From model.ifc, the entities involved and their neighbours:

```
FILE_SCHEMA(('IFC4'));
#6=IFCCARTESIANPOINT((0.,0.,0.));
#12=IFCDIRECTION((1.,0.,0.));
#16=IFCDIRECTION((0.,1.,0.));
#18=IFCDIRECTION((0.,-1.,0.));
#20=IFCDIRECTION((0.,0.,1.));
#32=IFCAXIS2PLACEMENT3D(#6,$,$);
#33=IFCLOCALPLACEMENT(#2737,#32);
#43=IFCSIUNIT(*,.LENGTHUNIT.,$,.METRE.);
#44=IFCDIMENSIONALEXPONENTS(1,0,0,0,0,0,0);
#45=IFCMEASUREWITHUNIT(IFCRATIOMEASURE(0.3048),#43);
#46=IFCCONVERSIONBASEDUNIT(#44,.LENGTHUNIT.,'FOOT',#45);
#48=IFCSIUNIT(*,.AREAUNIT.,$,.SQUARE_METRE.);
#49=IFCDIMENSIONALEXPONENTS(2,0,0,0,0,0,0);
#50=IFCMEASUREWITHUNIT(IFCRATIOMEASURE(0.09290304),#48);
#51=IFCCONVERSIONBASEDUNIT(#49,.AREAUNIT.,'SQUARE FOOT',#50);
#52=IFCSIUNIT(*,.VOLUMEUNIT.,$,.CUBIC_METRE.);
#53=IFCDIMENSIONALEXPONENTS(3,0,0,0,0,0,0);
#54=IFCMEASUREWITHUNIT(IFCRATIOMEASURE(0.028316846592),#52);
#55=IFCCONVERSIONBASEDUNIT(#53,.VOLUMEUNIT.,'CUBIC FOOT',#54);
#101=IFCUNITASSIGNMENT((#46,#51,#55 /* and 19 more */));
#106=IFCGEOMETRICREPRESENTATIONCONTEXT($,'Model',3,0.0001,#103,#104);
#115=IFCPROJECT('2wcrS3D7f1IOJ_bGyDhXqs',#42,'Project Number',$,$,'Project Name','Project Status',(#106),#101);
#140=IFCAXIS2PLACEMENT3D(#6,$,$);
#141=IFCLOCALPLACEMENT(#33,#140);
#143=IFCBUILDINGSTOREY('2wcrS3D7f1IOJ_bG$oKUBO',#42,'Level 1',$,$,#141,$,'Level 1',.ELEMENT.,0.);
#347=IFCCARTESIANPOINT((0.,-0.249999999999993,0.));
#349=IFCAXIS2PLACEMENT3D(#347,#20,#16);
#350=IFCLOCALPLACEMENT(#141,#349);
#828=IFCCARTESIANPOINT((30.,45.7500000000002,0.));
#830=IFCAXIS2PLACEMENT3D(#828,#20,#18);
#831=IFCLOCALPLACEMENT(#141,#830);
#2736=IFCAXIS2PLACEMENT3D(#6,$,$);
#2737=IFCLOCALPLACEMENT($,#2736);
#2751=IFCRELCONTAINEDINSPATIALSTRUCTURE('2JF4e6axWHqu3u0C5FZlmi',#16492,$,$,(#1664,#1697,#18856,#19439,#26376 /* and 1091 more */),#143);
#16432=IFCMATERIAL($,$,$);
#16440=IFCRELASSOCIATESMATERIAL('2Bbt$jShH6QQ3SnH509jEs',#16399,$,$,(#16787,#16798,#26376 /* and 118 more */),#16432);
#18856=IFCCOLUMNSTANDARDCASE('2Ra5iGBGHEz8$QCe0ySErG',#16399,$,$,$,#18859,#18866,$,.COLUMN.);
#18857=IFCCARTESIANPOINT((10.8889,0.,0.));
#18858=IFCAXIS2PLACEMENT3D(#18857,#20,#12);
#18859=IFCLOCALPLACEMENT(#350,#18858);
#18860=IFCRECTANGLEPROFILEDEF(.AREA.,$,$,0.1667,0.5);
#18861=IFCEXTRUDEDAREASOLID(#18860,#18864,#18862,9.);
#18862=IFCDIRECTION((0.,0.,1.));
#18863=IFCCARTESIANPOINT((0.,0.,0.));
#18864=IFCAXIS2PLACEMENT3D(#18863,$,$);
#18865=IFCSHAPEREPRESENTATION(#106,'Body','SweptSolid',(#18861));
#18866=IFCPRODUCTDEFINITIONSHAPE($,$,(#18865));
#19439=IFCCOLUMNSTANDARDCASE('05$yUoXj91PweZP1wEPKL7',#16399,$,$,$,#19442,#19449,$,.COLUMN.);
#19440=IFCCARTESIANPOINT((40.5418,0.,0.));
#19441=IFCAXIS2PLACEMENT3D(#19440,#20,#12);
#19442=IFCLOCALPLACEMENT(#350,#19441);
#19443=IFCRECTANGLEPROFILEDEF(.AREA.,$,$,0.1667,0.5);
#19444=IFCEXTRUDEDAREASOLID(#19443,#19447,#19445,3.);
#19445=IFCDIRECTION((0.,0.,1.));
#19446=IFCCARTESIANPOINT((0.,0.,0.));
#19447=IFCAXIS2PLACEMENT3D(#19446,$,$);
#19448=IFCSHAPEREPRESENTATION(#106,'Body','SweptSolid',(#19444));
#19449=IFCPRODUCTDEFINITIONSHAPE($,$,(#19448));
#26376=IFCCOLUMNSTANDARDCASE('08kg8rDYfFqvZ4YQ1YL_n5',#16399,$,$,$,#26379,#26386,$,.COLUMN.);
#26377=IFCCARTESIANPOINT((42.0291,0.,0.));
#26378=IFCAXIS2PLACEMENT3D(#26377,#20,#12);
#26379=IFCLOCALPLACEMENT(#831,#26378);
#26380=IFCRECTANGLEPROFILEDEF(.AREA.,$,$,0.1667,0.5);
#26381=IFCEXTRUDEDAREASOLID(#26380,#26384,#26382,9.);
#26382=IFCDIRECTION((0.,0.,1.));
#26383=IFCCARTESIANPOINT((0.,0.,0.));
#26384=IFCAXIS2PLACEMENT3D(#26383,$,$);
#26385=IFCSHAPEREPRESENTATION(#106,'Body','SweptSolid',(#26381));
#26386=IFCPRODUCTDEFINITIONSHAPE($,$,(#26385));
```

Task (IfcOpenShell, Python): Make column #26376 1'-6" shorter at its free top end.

```python
import ifcopenshell
import ifcopenshell.util.unit

model = ifcopenshell.open("model.ifc")
unit_scale = ifcopenshell.util.unit.calculate_unit_scale(model)

member = model.by_guid("08kg8rDYfFqvZ4YQ1YL_n5")
change = -18 * 0.0254 / unit_scale

# The extrusion runs towards the end named, so only its depth changes.
body = next(r for r in member.Representation.Representations if r.RepresentationIdentifier == "Body")
solid = body.Items[0]
old_length = solid.Depth
solid.Depth += change

print(f"length {old_length:g} -> {solid.Depth:g}")

model.write("model-out.ifc")
```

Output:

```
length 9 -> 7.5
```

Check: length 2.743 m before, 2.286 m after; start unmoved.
